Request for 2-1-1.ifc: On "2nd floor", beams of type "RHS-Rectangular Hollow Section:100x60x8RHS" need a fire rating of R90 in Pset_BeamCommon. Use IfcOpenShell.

First a look at what the model holds.

```python
import ifcopenshell
import ifcopenshell.util.element

model = ifcopenshell.open("2-1-1.ifc")
print(model.schema)
storey = next(s for s in model.by_type("IfcBuildingStorey") if s.Name == "2nd floor")
beams = [e for e in ifcopenshell.util.element.get_decomposition(storey) if e.is_a("IfcBeam")]
seen = {}
for e in beams:
    element_type = ifcopenshell.util.element.get_type(e)
    key = (element_type.Name if element_type != e and element_type else None, ifcopenshell.util.element.get_pset(e, "Pset_BeamCommon", "FireRating"))
    seen[key] = seen.get(key, 0) + 1
for (name, value), count in sorted(seen.items(), key=str):
    print(count, "x", name, "|", value)
```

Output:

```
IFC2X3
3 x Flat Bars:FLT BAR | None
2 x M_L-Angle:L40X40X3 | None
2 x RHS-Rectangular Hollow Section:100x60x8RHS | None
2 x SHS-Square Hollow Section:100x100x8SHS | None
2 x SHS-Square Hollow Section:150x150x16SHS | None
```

```python
import ifcopenshell
import ifcopenshell.api.pset
import ifcopenshell.util.element

model = ifcopenshell.open("2-1-1.ifc")

storey = next(s for s in model.by_type("IfcBuildingStorey") if s.Name == "2nd floor")
beams = [e for e in ifcopenshell.util.element.get_decomposition(storey) if e.is_a("IfcBeam")]

count = 0
for e in beams:
    element_type = ifcopenshell.util.element.get_type(e)
    if element_type in (None, e) or element_type.Name != "RHS-Rectangular Hollow Section:100x60x8RHS":
        continue
    # add_pset returns the element's existing set when there is one.
    pset = ifcopenshell.api.pset.add_pset(model, product=e, name="Pset_BeamCommon")
    ifcopenshell.api.pset.edit_pset(model, pset=pset, properties={"FireRating": "R90"})
    count += 1

print(count, "beams updated")

model.write("2-1-1_updated.ifc")
```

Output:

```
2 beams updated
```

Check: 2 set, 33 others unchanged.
